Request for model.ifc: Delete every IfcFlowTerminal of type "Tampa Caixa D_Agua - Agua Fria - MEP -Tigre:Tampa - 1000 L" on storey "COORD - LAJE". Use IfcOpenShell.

First a look at what the model holds.

```python
import ifcopenshell
import ifcopenshell.util.element

model = ifcopenshell.open("model.ifc")
print(model.schema)
storey = next(s for s in model.by_type("IfcBuildingStorey") if s.Name == "COORD - LAJE")
terminals = [e for e in ifcopenshell.util.element.get_decomposition(storey) if e.is_a("IfcFlowTerminal")]
seen = {}
for e in terminals:
    element_type = ifcopenshell.util.element.get_type(e)
    name = element_type.Name if element_type not in (None, e) else None
    seen[name] = seen.get(name, 0) + 1
for name, count in sorted(seen.items(), key=str):
    print(count, "x", name)
```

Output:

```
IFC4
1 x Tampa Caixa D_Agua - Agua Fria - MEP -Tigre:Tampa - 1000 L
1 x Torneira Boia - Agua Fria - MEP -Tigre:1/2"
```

```python
import ifcopenshell
import ifcopenshell.api.root
import ifcopenshell.util.element

model = ifcopenshell.open("model.ifc")

storey = next(s for s in model.by_type("IfcBuildingStorey") if s.Name == "COORD - LAJE")
terminals = [e for e in ifcopenshell.util.element.get_decomposition(storey) if e.is_a("IfcFlowTerminal")]
targets = [e for e in terminals if (t := ifcopenshell.util.element.get_type(e)) not in (None, e) and t.Name == "Tampa Caixa D_Agua - Agua Fria - MEP -Tigre:Tampa - 1000 L"]

for e in targets:
    ifcopenshell.api.root.remove_product(model, product=e)
print(len(targets), "removed")

model.write("model_rev.ifc")
```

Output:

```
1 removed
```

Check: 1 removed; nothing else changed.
